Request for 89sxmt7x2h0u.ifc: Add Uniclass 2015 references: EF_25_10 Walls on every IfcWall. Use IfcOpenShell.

First a look at what the model holds.

```python
import ifcopenshell

model = ifcopenshell.open("89sxmt7x2h0u.ifc")
print(model.schema)
print("classifications:", [c.Name for c in model.by_type("IfcClassification")])
for ifc_class in ("IfcDoor", "IfcRoof", "IfcStair", "IfcWall", "IfcWindow"):
    print(ifc_class, len(model.by_type(ifc_class)))
```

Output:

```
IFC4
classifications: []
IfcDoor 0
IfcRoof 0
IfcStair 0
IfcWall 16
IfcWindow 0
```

```python
import ifcopenshell
import ifcopenshell.api.classification

model = ifcopenshell.open("89sxmt7x2h0u.ifc")

system = ifcopenshell.api.classification.add_classification(model, classification="Uniclass 2015")

codes = {
    "IfcWall": ("EF_25_10", "Walls"),
}
for ifc_class, (code, name) in codes.items():
    products = model.by_type(ifc_class)
    ifcopenshell.api.classification.add_reference(
        model, products=products, classification=system, identification=code, name=name
    )
    print(code, len(products))

model.write("89sxmt7x2h0u_edited.ifc")
```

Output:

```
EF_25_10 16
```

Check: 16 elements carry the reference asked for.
